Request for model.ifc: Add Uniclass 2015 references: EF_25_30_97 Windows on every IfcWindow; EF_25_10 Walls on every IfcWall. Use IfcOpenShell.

First a look at what the model holds.

```python
import ifcopenshell

model = ifcopenshell.open("model.ifc")
print(model.schema)
print("classifications:", [c.Name for c in model.by_type("IfcClassification")])
for ifc_class in ("IfcDoor", "IfcRoof", "IfcStair", "IfcWall", "IfcWindow"):
    print(ifc_class, len(model.by_type(ifc_class)))
```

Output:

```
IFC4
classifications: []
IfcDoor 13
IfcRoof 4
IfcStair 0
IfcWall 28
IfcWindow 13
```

```python
import ifcopenshell
import ifcopenshell.api.classification

model = ifcopenshell.open("model.ifc")

system = ifcopenshell.api.classification.add_classification(model, classification="Uniclass 2015")

codes = {
    "IfcWindow": ("EF_25_30_97", "Windows"),
    "IfcWall": ("EF_25_10", "Walls"),
}
for ifc_class, (code, name) in codes.items():
    products = model.by_type(ifc_class)
    ifcopenshell.api.classification.add_reference(
        model, products=products, classification=system, identification=code, name=name
    )
    print(code, len(products))

model.write("model_edited.ifc")
```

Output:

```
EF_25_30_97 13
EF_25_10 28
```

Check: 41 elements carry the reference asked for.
